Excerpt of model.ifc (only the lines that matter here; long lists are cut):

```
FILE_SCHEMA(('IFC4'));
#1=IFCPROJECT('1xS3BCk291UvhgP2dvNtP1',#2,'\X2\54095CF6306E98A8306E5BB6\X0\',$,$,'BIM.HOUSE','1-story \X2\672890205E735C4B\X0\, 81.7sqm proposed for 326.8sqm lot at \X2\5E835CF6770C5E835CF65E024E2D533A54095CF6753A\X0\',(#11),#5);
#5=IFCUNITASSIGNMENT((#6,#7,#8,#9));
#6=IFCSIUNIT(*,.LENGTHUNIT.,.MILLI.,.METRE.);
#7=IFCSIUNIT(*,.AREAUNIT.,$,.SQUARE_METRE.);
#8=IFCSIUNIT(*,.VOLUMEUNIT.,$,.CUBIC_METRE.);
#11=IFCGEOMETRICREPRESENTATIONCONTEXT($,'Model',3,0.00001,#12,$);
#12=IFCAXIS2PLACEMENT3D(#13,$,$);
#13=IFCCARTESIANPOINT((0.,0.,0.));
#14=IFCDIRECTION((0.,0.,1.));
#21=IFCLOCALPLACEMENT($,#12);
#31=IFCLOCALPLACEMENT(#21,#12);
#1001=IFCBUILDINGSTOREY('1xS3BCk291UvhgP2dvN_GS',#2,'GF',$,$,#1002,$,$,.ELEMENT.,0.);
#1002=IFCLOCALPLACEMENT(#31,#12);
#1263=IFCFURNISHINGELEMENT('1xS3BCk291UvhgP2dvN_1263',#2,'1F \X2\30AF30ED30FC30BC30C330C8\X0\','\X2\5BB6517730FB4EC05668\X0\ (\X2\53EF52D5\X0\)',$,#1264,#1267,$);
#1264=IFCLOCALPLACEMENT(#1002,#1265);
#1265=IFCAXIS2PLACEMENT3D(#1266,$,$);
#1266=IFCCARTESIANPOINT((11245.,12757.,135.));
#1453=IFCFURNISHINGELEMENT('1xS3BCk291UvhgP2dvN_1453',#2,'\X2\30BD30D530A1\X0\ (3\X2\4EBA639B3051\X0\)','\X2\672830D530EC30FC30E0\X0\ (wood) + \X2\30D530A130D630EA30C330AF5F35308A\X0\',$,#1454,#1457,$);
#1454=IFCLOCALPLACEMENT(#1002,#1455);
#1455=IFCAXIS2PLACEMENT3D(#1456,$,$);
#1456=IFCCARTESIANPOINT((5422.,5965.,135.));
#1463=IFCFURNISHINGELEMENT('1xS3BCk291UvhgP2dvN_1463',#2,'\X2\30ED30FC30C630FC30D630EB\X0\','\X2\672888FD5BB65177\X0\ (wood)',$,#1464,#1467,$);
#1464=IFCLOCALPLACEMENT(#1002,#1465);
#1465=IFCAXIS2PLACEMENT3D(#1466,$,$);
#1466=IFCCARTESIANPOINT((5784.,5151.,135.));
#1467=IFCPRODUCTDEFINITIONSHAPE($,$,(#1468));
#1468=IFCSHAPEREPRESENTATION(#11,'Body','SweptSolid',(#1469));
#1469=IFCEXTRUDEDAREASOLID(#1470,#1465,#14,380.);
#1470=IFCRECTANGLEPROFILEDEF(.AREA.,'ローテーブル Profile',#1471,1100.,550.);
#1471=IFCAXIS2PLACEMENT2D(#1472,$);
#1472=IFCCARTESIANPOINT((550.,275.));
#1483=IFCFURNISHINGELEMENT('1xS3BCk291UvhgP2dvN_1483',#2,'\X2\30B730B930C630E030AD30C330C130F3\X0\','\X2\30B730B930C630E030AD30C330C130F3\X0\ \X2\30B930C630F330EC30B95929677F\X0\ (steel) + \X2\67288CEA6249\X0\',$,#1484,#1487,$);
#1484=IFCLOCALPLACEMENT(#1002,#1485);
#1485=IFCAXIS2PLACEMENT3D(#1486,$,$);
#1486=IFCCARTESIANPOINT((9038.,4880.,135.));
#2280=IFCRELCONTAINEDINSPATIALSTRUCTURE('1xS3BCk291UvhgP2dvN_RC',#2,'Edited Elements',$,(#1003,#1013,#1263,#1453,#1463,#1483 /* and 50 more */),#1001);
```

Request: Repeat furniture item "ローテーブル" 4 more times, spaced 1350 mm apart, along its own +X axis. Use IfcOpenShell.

```python
import ifcopenshell
import ifcopenshell.api.geometry
import ifcopenshell.api.root
import ifcopenshell.util.element
import ifcopenshell.util.placement

model = ifcopenshell.open("model.ifc")


def reuse_history(source, copy):
    """copy_class also copies each property set's owner history, people and application; keep the originals."""
    for rel in copy.IsDefinedBy:
        if rel.is_a("IfcRelDefinesByProperties") and (history := rel.RelatingPropertyDefinition.OwnerHistory):
            rel.RelatingPropertyDefinition.OwnerHistory = source.OwnerHistory
            ifcopenshell.util.element.remove_deep2(model, history)


source = model.by_guid("1xS3BCk291UvhgP2dvN_1463")
base = ifcopenshell.util.placement.get_local_placement(source.ObjectPlacement)
step = base[:3, 0] * 1350.0

for i in range(1, 5):
    copy = ifcopenshell.api.root.copy_class(model, product=source)
    copy.Representation = ifcopenshell.util.element.copy_deep(
        model, source.Representation, exclude=["IfcGeometricRepresentationContext", "IfcRepresentationMap"]
    )
    reuse_history(source, copy)
    matrix = base.copy()
    matrix[:3, 3] += i * step
    print("added at", matrix[:3, 3].round(3) + 0.0)
    ifcopenshell.api.geometry.edit_object_placement(model, product=copy, matrix=matrix, is_si=False)

model.write("model_v2.ifc")
```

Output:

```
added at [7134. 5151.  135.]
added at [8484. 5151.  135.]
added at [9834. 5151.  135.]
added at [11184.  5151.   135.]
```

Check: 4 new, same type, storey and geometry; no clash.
